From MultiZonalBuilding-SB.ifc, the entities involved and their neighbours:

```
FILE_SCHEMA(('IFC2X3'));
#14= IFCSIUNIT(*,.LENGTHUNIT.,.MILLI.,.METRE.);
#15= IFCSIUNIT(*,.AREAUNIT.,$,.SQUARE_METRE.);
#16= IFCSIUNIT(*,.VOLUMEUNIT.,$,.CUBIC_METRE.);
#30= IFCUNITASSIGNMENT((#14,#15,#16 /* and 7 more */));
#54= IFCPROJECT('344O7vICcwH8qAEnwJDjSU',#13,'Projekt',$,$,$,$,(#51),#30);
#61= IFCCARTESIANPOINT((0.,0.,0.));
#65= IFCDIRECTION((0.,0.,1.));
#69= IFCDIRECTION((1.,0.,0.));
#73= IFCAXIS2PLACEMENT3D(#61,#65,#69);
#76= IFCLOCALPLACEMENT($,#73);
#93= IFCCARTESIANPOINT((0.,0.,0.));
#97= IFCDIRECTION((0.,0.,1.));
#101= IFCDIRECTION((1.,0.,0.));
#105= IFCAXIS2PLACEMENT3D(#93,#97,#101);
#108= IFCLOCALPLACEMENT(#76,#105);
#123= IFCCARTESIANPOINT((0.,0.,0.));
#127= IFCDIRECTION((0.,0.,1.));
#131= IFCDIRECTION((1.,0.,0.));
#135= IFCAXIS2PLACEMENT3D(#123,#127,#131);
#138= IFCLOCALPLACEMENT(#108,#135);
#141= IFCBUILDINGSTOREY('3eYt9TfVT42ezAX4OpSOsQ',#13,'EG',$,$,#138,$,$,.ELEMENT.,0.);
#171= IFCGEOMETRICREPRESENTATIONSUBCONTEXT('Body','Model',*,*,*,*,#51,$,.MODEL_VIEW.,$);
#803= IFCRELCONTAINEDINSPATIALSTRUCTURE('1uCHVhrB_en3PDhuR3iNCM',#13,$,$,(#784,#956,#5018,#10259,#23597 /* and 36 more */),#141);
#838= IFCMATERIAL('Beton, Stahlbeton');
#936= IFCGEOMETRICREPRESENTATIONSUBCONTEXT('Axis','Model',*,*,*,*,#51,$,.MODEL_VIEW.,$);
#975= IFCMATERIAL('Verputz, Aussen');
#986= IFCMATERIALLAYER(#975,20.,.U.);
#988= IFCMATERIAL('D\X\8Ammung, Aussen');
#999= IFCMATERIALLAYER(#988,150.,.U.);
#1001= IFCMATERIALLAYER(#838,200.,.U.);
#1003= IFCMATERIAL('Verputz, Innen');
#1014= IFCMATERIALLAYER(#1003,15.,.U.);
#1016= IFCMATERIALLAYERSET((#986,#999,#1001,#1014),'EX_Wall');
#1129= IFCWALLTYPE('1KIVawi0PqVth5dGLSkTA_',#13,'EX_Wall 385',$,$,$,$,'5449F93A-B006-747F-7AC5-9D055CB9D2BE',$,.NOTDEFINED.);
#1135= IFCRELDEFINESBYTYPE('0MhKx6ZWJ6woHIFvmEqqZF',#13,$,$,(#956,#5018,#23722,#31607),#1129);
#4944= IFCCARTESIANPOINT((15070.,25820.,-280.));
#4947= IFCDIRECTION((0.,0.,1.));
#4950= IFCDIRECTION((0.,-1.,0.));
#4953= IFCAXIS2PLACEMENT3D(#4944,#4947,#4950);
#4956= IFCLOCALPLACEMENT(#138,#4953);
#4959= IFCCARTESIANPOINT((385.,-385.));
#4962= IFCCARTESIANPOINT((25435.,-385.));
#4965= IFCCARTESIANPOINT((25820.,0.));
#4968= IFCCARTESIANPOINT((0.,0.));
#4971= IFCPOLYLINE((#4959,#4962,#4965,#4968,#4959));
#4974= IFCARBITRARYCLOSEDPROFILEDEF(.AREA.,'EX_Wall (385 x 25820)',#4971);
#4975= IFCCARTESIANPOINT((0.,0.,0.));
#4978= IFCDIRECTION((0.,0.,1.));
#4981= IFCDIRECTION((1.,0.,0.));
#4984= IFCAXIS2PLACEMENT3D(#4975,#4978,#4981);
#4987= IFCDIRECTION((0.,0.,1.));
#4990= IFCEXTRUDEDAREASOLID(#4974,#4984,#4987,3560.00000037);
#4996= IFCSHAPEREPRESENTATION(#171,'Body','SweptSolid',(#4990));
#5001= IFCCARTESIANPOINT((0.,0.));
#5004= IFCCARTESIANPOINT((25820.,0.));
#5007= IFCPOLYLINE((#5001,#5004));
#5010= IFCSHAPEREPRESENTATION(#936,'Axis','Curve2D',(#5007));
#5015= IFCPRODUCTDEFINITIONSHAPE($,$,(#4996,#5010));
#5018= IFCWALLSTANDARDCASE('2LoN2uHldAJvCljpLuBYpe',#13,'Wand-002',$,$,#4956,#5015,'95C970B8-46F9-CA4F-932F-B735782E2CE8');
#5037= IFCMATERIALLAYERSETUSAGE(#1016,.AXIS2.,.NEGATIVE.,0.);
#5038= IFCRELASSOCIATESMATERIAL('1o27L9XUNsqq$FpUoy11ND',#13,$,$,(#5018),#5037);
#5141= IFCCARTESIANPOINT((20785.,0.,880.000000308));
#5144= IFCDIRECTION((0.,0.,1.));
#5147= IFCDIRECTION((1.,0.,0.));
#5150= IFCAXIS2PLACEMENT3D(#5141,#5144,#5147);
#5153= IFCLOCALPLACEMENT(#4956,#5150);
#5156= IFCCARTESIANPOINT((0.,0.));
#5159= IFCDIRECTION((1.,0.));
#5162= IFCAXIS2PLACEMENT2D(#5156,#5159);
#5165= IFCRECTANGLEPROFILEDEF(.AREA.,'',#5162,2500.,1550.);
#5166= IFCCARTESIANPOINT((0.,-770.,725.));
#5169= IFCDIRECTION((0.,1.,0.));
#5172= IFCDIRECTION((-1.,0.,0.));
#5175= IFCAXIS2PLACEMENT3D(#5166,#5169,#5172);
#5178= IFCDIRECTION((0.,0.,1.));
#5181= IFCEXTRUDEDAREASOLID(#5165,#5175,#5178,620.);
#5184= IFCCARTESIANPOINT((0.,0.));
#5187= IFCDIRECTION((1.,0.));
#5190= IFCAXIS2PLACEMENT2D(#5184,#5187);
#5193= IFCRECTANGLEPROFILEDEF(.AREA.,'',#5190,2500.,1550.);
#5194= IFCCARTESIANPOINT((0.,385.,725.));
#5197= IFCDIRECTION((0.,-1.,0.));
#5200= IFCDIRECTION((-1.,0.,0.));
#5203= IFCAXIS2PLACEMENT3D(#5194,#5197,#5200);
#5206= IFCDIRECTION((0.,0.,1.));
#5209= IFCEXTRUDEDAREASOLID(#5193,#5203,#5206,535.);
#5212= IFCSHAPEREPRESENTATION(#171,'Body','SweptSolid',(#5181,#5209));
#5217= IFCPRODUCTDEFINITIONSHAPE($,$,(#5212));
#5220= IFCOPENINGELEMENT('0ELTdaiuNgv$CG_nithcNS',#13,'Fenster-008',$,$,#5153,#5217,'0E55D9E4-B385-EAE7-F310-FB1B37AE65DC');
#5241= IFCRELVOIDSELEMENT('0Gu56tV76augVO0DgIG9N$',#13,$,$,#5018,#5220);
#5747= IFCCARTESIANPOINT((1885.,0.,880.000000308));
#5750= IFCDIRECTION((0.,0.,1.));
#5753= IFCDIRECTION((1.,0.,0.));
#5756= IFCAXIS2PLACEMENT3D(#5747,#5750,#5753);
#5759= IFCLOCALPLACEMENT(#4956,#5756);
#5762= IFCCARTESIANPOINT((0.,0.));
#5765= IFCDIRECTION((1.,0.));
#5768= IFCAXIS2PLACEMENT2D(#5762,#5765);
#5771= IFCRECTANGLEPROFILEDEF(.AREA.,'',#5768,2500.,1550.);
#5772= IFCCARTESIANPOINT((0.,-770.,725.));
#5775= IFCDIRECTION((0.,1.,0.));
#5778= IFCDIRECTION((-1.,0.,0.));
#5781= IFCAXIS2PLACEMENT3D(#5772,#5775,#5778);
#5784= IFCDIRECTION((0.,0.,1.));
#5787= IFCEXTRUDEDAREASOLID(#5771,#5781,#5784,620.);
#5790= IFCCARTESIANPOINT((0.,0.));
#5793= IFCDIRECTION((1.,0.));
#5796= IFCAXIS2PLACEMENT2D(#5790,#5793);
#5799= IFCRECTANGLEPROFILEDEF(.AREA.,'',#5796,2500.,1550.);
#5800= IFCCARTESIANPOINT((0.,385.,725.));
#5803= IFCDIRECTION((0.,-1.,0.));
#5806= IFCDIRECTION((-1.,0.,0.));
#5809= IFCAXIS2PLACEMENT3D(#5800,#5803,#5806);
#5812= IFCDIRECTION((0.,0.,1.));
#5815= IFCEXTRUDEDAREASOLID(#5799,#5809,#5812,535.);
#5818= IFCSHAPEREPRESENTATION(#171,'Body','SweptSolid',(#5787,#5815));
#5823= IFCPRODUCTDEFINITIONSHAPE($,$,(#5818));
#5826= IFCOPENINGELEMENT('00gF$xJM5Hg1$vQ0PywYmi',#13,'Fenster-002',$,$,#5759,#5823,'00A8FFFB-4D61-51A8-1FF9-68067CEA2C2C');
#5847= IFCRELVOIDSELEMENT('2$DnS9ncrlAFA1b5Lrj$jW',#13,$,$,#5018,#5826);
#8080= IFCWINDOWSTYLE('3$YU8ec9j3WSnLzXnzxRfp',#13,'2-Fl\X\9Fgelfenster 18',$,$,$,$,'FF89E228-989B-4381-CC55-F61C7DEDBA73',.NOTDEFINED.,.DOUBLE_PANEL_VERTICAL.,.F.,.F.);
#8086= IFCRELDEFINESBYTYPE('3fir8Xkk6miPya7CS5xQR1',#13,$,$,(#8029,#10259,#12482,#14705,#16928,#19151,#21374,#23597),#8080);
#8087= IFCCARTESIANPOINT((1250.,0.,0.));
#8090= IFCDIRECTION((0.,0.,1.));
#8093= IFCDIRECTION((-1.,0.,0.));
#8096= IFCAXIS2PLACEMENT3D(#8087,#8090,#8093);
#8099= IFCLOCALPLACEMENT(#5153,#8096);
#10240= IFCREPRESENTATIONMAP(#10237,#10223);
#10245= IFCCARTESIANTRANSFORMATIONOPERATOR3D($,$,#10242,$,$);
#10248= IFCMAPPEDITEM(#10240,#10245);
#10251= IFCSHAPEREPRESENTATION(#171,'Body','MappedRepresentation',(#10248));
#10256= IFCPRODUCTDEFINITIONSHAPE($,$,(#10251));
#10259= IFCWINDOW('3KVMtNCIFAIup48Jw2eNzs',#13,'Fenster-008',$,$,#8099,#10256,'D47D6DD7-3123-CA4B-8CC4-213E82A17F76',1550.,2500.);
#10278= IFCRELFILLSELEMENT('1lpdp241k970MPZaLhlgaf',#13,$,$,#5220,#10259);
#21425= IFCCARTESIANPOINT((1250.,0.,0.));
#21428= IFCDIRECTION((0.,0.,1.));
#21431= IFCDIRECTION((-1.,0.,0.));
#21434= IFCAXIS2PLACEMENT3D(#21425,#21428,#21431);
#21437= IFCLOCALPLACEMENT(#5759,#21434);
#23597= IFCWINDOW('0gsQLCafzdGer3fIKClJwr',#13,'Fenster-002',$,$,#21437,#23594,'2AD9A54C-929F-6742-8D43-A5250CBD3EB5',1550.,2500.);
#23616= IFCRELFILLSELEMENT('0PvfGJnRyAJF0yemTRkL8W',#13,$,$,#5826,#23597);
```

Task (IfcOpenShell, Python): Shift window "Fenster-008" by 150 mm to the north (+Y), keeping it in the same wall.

```python
import ifcopenshell
import ifcopenshell.api.geometry
import ifcopenshell.util.placement
import ifcopenshell.util.unit

model = ifcopenshell.open("MultiZonalBuilding-SB.ifc")
unit_scale = ifcopenshell.util.unit.calculate_unit_scale(model)

window = model.by_guid("3KVMtNCIFAIup48Jw2eNzs")
opening = window.FillsVoids[0].RelatingOpeningElement
wall = opening.VoidsElements[0].RelatingBuildingElement

wall_matrix = ifcopenshell.util.placement.get_local_placement(wall.ObjectPlacement)
shift = wall_matrix[:3, 0] * -0.15 / unit_scale
before = ifcopenshell.util.placement.get_local_placement(window.ObjectPlacement)[:3, 3].copy()

# The window is placed relative to its opening, so it follows when the opening moves.
matrix = ifcopenshell.util.placement.get_local_placement(opening.ObjectPlacement)
matrix[:3, 3] += shift
ifcopenshell.api.geometry.edit_object_placement(
    model, product=opening, matrix=matrix, is_si=False, should_transform_children=True
)

after = ifcopenshell.util.placement.get_local_placement(window.ObjectPlacement)[:3, 3]
print("window moved by", (after - before).round(3) + 0.0)

model.write("MultiZonalBuilding-SB_edited.ifc")
```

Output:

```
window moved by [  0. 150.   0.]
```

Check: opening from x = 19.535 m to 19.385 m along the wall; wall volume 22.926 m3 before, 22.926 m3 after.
